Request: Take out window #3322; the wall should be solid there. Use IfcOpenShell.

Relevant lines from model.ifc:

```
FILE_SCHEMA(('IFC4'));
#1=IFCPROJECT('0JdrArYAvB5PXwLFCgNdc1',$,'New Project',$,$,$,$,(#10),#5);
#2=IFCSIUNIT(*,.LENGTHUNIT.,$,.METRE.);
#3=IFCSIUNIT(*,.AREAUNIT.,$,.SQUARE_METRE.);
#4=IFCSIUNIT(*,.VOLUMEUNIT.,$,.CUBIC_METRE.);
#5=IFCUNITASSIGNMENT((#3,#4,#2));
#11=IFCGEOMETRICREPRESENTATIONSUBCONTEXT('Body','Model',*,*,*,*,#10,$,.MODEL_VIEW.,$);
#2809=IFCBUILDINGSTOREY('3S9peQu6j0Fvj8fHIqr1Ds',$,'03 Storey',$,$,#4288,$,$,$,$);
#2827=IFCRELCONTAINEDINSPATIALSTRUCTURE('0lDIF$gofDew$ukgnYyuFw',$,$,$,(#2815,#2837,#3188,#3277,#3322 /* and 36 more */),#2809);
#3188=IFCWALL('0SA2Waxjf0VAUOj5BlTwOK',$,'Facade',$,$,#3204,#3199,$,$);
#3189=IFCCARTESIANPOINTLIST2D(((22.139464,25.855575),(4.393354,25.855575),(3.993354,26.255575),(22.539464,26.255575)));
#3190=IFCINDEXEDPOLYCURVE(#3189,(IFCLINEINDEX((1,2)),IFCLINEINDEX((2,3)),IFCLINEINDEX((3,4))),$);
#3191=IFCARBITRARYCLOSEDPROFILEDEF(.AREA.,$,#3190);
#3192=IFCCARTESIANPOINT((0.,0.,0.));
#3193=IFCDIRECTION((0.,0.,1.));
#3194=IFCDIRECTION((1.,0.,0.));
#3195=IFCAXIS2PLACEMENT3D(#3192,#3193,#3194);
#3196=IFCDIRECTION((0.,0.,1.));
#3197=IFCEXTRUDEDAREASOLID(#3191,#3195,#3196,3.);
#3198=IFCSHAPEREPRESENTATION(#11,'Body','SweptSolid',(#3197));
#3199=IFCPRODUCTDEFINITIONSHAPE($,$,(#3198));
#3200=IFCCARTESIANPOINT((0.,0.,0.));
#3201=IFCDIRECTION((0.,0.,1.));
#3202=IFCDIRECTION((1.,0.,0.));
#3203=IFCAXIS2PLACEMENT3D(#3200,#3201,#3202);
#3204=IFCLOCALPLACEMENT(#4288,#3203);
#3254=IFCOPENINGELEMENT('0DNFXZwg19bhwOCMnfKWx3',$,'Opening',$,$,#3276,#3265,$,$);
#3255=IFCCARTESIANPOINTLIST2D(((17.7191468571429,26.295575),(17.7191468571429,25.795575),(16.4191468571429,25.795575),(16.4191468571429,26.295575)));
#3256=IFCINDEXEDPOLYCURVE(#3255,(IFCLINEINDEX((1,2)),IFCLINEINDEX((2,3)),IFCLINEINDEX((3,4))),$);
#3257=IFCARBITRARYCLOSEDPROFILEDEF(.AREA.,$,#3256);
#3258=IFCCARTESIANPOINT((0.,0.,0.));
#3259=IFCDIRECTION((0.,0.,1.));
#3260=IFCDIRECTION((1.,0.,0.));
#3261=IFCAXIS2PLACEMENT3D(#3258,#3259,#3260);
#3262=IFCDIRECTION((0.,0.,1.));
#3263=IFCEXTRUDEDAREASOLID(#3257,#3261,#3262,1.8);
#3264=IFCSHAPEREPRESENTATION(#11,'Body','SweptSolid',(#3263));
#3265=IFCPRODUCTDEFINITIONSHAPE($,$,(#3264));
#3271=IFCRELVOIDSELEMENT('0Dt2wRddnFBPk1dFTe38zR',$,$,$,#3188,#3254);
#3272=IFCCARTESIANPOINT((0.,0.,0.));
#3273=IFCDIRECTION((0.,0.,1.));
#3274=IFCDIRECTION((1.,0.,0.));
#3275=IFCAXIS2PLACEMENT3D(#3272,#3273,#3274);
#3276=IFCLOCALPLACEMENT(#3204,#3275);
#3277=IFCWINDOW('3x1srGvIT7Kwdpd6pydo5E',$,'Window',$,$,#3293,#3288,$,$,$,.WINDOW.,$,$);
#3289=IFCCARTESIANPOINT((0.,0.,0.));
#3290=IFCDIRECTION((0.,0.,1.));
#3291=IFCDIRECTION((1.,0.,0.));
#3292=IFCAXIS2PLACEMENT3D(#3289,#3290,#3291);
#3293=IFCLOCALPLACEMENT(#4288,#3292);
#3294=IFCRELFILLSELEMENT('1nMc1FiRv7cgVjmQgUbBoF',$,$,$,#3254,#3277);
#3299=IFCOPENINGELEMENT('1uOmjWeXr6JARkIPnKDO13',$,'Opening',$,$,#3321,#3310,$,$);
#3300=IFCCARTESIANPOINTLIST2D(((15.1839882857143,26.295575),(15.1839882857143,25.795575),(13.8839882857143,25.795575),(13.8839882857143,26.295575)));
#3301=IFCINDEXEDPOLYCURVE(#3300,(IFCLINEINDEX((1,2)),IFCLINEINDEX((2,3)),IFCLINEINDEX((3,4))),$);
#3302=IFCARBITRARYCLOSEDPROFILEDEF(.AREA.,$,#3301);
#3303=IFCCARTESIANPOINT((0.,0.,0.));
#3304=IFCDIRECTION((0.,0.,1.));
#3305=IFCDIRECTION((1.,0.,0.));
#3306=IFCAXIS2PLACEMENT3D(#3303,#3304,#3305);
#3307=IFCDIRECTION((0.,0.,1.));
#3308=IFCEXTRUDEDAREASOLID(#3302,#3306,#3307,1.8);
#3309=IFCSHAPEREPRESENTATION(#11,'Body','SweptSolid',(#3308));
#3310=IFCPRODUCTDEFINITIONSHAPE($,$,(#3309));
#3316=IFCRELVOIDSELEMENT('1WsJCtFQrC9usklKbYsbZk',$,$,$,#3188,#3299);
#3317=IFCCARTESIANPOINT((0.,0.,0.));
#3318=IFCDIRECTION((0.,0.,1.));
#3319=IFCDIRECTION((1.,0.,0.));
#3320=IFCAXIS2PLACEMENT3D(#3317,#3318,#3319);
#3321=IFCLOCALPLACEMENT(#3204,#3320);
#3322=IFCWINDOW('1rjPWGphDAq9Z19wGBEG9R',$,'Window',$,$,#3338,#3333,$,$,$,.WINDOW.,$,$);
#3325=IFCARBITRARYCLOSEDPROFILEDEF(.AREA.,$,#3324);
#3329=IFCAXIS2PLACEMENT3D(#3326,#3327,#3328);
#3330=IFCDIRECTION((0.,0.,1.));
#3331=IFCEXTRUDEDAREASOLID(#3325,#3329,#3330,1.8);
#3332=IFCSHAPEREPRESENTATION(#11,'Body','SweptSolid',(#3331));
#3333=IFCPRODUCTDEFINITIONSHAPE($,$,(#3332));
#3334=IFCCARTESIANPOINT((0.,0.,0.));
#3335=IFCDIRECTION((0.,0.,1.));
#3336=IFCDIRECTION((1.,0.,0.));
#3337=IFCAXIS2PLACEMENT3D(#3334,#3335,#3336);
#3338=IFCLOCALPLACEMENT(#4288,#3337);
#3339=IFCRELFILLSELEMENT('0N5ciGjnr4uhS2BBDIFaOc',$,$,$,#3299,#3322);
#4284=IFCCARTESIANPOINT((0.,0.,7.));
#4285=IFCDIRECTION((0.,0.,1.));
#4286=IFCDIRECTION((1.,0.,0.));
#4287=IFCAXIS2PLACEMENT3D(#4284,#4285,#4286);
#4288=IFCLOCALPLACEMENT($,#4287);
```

```python
import ifcopenshell
import ifcopenshell.api.feature
import ifcopenshell.api.root
import ifcopenshell.geom
import ifcopenshell.util.shape

model = ifcopenshell.open("model.ifc")
settings = ifcopenshell.geom.settings()


def volume(element):
    """Net volume in cubic metres, openings subtracted."""
    shape = ifcopenshell.geom.create_shape(settings, element)
    return ifcopenshell.util.shape.get_volume(shape.geometry)


window = model.by_guid("1rjPWGphDAq9Z19wGBEG9R")
opening = window.FillsVoids[0].RelatingOpeningElement
wall = opening.VoidsElements[0].RelatingBuildingElement
before = volume(wall)

ifcopenshell.api.root.remove_product(model, product=window)
ifcopenshell.api.feature.remove_feature(model, feature=opening)

after = volume(wall)

print(f"wall volume {before:.3f} -> {after:.3f} m3")

model.write("model_v2.ifc")
```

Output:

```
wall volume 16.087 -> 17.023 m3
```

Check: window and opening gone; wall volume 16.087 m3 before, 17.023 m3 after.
